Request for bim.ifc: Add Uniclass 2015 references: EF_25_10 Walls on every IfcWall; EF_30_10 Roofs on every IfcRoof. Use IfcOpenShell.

First a look at what the model holds.

```python
import ifcopenshell

model = ifcopenshell.open("bim.ifc")
print(model.schema)
print("classifications:", [c.Name for c in model.by_type("IfcClassification")])
for ifc_class in ("IfcDoor", "IfcRoof", "IfcStair", "IfcWall", "IfcWindow"):
    print(ifc_class, len(model.by_type(ifc_class)))
```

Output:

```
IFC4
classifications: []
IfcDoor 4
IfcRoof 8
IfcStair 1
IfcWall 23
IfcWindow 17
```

```python
import ifcopenshell
import ifcopenshell.api.classification

model = ifcopenshell.open("bim.ifc")

system = ifcopenshell.api.classification.add_classification(model, classification="Uniclass 2015")

codes = {
    "IfcWall": ("EF_25_10", "Walls"),
    "IfcRoof": ("EF_30_10", "Roofs"),
}
for ifc_class, (code, name) in codes.items():
    products = model.by_type(ifc_class)
    ifcopenshell.api.classification.add_reference(
        model, products=products, classification=system, identification=code, name=name
    )
    print(code, len(products))

model.write("bim_edited.ifc")
```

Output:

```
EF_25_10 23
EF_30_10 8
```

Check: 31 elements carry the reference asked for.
